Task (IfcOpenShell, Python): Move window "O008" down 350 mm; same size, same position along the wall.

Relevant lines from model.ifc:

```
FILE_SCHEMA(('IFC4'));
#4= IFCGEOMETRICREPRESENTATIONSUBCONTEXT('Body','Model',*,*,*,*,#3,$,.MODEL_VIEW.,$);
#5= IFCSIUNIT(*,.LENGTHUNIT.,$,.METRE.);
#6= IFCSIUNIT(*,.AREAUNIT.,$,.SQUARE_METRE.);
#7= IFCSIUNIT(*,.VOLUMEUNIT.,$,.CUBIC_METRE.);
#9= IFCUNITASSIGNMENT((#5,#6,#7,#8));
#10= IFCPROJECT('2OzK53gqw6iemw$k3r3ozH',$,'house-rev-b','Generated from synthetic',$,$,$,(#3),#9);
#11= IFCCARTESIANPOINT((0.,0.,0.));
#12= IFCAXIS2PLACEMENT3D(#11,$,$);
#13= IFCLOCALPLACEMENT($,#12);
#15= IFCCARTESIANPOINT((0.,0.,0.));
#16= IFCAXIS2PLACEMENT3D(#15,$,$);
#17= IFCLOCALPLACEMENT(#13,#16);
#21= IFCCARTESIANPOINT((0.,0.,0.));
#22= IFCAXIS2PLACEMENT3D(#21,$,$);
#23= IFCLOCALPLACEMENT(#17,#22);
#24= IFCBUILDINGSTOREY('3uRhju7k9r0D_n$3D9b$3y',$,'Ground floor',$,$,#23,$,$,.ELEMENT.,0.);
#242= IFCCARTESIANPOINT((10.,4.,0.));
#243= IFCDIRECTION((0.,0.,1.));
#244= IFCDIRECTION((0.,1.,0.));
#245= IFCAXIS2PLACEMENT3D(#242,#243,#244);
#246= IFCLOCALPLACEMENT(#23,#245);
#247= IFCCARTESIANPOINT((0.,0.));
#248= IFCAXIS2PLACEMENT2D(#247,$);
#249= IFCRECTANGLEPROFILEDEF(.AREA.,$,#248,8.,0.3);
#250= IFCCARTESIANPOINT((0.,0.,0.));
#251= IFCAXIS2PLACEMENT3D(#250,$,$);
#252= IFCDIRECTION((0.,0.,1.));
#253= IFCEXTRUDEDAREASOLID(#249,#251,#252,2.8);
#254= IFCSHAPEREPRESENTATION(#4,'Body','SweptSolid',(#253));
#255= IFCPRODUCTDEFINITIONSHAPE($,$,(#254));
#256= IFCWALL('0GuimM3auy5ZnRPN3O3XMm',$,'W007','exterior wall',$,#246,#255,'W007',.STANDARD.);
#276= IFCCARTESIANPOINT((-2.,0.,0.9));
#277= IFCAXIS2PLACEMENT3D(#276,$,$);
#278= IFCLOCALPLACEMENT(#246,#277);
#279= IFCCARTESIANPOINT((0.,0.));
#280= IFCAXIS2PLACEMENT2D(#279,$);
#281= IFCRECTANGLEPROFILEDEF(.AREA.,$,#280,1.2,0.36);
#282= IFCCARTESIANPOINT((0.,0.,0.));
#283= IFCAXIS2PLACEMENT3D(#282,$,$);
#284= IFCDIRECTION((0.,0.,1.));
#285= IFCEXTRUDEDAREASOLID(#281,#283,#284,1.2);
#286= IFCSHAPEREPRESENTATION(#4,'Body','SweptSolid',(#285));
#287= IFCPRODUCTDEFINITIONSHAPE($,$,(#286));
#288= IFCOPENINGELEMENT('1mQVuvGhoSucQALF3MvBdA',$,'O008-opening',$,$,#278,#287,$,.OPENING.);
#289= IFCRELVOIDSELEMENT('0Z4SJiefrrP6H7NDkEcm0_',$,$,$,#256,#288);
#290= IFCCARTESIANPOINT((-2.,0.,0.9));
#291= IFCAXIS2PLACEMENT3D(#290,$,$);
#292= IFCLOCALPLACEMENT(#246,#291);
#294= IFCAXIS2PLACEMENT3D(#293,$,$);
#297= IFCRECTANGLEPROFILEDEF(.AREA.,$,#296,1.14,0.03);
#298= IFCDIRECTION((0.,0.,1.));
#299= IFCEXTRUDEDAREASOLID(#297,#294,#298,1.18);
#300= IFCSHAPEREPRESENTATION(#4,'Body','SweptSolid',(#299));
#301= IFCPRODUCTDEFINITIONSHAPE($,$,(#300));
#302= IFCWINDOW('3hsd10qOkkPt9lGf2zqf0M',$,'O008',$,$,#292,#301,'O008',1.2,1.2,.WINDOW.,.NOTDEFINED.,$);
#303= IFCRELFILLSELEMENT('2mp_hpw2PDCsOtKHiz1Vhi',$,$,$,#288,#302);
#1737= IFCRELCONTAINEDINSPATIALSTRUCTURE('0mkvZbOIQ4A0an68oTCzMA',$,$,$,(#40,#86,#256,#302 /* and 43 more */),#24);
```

```python
import numpy as np
import ifcopenshell
import ifcopenshell.api.geometry
import ifcopenshell.util.placement
import ifcopenshell.util.unit

model = ifcopenshell.open("model.ifc")
unit_scale = ifcopenshell.util.unit.calculate_unit_scale(model)

window = model.by_guid("3hsd10qOkkPt9lGf2zqf0M")
opening = window.FillsVoids[0].RelatingOpeningElement
dz = -0.35 / unit_scale

shift = np.array([0.0, 0.0, dz])
# The window is not placed relative to its opening, so move both.
for product in (opening, window):
    matrix = ifcopenshell.util.placement.get_local_placement(product.ObjectPlacement)
    matrix[:3, 3] += shift
    ifcopenshell.api.geometry.edit_object_placement(model, product=product, matrix=matrix, is_si=False)

print(f"moved by {dz * unit_scale:+.3f} m")

model.write("model_edited.ifc")
```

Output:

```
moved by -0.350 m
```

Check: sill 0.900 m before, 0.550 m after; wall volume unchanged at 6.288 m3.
